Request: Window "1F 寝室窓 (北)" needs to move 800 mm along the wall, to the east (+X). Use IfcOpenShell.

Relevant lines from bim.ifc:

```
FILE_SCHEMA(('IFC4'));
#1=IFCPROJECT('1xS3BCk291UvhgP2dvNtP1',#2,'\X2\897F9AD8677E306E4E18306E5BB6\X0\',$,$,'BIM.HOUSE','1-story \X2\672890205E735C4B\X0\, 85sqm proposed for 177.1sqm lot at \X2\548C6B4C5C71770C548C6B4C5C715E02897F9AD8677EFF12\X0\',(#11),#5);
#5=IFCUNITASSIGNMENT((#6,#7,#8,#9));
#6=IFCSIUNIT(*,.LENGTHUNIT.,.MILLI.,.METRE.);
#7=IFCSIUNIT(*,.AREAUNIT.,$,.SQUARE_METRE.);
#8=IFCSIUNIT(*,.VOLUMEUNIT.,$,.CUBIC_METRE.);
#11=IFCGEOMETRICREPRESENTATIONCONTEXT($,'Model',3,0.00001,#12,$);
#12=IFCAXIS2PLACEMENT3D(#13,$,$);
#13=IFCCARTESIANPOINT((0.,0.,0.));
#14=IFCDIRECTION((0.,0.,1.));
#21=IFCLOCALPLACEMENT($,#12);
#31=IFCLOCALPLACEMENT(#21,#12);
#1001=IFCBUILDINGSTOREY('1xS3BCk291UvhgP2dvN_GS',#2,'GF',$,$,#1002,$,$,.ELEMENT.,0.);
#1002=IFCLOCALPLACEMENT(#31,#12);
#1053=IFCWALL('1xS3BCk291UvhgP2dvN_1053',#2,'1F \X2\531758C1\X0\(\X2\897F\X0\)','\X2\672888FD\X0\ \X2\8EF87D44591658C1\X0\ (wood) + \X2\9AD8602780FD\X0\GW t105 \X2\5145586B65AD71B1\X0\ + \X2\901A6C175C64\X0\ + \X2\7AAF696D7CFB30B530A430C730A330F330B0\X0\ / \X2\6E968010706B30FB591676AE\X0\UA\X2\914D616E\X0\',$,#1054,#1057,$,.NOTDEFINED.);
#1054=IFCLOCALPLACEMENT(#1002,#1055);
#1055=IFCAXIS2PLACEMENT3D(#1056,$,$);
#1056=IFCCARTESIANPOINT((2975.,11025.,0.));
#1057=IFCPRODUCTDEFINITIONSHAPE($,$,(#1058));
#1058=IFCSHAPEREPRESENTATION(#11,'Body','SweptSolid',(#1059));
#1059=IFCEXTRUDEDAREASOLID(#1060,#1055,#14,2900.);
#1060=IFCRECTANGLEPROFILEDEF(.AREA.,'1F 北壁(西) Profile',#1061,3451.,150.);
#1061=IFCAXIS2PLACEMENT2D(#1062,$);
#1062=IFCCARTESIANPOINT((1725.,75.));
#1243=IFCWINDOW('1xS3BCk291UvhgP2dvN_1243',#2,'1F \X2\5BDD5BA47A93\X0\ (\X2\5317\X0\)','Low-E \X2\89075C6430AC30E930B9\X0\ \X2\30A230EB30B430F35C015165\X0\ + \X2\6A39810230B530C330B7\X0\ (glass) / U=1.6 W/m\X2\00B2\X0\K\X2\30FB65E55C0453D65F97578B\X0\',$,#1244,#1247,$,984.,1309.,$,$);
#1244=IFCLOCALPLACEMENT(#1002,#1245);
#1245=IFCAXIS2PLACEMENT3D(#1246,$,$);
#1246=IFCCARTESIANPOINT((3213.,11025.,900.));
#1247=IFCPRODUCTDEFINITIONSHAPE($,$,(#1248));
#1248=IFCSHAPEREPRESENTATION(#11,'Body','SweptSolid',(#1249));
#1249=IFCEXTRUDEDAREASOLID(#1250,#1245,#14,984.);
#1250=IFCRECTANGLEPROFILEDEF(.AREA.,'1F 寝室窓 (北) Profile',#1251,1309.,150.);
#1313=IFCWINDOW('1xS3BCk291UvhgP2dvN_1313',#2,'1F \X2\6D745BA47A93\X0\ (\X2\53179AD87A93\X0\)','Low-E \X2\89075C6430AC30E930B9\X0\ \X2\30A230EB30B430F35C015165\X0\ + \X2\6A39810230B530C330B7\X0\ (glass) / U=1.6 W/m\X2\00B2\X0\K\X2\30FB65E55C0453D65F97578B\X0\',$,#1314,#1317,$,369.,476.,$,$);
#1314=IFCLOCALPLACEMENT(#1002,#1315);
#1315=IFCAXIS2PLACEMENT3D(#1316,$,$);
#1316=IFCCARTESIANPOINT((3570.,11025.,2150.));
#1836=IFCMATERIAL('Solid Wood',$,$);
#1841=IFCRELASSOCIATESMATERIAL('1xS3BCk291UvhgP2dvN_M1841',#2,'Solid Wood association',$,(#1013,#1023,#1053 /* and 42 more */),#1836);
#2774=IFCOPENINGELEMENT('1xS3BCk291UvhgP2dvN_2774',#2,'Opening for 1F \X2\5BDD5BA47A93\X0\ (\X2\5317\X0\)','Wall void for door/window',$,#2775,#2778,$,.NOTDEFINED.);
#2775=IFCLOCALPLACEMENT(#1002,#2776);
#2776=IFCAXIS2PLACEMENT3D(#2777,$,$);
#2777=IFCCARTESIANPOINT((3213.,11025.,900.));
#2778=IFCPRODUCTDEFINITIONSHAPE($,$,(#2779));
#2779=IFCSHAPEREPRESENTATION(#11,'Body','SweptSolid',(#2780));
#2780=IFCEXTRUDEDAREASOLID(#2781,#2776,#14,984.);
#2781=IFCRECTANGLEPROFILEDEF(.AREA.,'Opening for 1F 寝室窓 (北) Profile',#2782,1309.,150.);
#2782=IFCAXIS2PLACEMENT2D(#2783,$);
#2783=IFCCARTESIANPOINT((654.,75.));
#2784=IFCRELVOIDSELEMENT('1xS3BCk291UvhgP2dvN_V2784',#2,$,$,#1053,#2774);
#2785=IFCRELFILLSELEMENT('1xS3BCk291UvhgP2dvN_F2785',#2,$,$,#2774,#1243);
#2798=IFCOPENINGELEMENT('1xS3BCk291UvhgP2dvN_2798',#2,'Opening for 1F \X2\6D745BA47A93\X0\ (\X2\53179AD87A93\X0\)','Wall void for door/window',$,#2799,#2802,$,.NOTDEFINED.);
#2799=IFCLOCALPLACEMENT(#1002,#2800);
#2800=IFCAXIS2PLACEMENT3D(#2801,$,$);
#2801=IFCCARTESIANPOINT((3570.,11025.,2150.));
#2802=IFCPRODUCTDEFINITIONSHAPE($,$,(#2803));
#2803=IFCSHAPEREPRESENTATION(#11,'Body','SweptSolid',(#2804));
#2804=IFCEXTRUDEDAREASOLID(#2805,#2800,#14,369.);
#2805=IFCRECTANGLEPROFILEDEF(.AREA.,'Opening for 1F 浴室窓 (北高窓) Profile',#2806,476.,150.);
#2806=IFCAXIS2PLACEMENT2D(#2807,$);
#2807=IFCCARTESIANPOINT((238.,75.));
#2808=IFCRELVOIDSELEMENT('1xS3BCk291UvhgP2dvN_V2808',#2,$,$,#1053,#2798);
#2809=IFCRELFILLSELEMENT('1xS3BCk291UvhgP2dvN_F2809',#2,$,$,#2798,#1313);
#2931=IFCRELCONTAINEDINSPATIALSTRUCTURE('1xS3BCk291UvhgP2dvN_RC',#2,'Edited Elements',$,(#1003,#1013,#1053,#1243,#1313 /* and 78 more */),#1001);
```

```python
import ifcopenshell
import ifcopenshell.api.geometry
import ifcopenshell.util.placement

model = ifcopenshell.open("bim.ifc")

window = model.by_id(1243)
opening = window.FillsVoids[0].RelatingOpeningElement
wall = opening.VoidsElements[0].RelatingBuildingElement

wall_matrix = ifcopenshell.util.placement.get_local_placement(wall.ObjectPlacement)
shift = wall_matrix[:3, 0] * 800.0
before = ifcopenshell.util.placement.get_local_placement(window.ObjectPlacement)[:3, 3].copy()

# The window is not placed relative to its opening, so move both.
for product in (opening, window):
    matrix = ifcopenshell.util.placement.get_local_placement(product.ObjectPlacement)
    matrix[:3, 3] += shift
    ifcopenshell.api.geometry.edit_object_placement(model, product=product, matrix=matrix, is_si=False)

after = ifcopenshell.util.placement.get_local_placement(window.ObjectPlacement)[:3, 3]
print("window moved by", (after - before).round(3) + 0.0)

model.write("bim_edited.ifc")
```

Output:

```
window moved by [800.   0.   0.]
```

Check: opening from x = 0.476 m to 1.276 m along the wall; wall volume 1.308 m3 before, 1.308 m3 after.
